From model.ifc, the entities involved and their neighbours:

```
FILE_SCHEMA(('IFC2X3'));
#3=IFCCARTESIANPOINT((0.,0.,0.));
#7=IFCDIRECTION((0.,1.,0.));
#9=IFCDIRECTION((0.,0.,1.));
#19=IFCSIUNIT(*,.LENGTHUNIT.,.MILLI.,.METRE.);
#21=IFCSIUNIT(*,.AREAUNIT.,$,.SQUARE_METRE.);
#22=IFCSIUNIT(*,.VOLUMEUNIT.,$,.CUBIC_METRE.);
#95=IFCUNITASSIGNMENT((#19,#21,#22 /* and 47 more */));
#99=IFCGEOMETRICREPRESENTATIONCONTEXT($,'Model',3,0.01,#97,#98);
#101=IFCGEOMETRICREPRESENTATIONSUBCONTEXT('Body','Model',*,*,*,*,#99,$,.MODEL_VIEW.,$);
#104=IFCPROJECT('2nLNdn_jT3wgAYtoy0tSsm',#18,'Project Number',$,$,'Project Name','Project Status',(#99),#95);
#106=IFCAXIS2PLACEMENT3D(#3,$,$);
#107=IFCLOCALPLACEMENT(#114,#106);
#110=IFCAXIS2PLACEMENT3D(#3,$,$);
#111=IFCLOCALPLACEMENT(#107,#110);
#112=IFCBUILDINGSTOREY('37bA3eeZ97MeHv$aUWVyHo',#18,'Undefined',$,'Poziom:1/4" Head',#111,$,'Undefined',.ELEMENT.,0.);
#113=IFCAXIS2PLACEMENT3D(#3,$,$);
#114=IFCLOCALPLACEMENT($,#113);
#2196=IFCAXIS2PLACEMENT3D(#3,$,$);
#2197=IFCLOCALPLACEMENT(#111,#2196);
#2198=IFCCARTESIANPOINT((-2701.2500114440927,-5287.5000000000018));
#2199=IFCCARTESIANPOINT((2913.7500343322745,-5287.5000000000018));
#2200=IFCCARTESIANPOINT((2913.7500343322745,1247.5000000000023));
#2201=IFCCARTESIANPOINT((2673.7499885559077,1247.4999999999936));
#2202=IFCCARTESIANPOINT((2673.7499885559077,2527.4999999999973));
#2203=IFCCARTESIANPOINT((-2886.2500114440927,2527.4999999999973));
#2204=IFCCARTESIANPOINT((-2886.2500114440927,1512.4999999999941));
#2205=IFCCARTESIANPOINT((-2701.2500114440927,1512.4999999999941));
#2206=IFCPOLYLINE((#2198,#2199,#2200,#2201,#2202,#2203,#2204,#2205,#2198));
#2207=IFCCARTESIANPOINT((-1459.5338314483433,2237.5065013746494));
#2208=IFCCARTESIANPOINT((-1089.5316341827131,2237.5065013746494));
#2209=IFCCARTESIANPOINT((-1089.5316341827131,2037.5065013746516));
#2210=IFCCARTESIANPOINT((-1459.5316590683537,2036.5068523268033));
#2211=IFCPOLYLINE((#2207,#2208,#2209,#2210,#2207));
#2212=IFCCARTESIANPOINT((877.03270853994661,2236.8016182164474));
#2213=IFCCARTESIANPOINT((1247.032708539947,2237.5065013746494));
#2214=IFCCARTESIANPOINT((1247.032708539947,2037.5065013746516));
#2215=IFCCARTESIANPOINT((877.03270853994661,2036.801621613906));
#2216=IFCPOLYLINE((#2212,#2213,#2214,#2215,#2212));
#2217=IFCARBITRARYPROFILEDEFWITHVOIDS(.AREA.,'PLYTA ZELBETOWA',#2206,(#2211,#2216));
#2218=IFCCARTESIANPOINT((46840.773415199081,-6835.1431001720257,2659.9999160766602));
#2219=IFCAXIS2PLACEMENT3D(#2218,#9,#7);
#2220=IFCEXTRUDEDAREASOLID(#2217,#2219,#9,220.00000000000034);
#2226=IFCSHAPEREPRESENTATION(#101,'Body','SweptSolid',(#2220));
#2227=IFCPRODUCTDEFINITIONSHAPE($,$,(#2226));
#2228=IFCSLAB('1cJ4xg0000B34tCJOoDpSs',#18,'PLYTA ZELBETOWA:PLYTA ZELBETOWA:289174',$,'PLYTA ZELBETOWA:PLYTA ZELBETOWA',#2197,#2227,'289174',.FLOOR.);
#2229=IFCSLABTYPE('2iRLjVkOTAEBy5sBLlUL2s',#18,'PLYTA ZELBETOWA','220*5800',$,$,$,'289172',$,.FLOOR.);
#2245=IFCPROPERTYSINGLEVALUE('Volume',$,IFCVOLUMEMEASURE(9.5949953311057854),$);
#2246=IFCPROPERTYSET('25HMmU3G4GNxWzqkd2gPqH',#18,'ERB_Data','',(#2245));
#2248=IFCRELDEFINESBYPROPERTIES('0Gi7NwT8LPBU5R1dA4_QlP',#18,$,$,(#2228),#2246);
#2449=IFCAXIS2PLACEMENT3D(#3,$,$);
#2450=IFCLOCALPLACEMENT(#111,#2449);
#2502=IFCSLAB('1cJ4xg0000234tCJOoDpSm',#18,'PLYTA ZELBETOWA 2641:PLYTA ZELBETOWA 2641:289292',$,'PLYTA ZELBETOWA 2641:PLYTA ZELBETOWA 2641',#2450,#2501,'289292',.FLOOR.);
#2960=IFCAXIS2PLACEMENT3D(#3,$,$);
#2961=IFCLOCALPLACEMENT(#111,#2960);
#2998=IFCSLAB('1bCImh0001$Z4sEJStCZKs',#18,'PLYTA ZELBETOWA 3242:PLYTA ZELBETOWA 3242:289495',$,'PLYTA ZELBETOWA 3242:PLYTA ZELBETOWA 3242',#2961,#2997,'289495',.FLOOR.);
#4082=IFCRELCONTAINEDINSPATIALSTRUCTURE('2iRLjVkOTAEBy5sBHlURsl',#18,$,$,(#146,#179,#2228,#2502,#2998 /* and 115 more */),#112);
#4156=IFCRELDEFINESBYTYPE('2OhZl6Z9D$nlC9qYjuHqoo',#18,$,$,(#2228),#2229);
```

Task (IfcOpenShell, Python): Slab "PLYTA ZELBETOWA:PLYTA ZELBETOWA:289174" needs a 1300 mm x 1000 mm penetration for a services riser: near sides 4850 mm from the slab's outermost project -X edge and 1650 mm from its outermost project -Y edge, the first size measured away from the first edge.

```python
import numpy as np
import ifcopenshell
import ifcopenshell.api.feature
import ifcopenshell.api.geometry
import ifcopenshell.api.pset
import ifcopenshell.api.root
import ifcopenshell.geom
import ifcopenshell.util.element
import ifcopenshell.util.placement
import ifcopenshell.util.representation
import ifcopenshell.util.shape
import ifcopenshell.util.unit

model = ifcopenshell.open("model.ifc")
unit_scale = ifcopenshell.util.unit.calculate_unit_scale(model)
volume_scale = ifcopenshell.util.unit.calculate_unit_scale(model, "VOLUMEUNIT")
settings = ifcopenshell.geom.settings()


def volume(element):
    """Net volume in cubic metres, openings subtracted."""
    shape = ifcopenshell.geom.create_shape(settings, element)
    return ifcopenshell.util.shape.get_volume(shape.geometry)


slab = model.by_id(2228)
before = volume(slab)

# Extent in the slab's own axes, in metres. The edges named are its -X and -Y sides.
slab_shape = ifcopenshell.geom.create_shape(settings, slab)
vertices = ifcopenshell.util.shape.get_vertices(slab_shape.geometry)
x_min, y_min, bottom = vertices.min(axis=0)
top = vertices[:, 2].max()

opening = ifcopenshell.api.root.create_entity(model, ifc_class="IfcOpeningElement", name="Services riser opening")
context = ifcopenshell.util.representation.get_context(model, "Model", "Body", "MODEL_VIEW")
width, depth = 1.3, 1
outline = [(0.0, 0.0), (width, 0.0), (width, depth), (0.0, depth), (0.0, 0.0)]
# Overshoot both faces by 50 mm so the cut is clean.
shape = ifcopenshell.api.geometry.add_slab_representation(
    model, context=context, depth=top - bottom + 0.1, polyline=outline
)
ifcopenshell.api.geometry.assign_representation(model, product=opening, representation=shape)

matrix = ifcopenshell.util.placement.get_local_placement(slab.ObjectPlacement)
matrix[:, 3] = matrix @ np.append(np.array([x_min + 4.85, y_min + 1.65, bottom - 0.05]) / unit_scale, 1.0)
ifcopenshell.api.geometry.edit_object_placement(model, product=opening, matrix=matrix, is_si=False)
ifcopenshell.api.feature.add_feature(model, feature=opening, element=slab)

after = volume(slab)

# Update the slab's stored quantities.
pset = model.by_id(ifcopenshell.util.element.get_pset(slab, "ERB_Data", should_inherit=False)["id"])
ifcopenshell.api.pset.edit_pset(model, pset=pset, properties={
    "Volume": model.create_entity("IfcVolumeMeasure", after / volume_scale),
})

print(f"slab volume {before:.3f} -> {after:.3f} m3")

model.write("model_updated.ifc")
```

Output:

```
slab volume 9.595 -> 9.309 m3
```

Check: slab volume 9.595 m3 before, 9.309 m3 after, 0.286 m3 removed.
